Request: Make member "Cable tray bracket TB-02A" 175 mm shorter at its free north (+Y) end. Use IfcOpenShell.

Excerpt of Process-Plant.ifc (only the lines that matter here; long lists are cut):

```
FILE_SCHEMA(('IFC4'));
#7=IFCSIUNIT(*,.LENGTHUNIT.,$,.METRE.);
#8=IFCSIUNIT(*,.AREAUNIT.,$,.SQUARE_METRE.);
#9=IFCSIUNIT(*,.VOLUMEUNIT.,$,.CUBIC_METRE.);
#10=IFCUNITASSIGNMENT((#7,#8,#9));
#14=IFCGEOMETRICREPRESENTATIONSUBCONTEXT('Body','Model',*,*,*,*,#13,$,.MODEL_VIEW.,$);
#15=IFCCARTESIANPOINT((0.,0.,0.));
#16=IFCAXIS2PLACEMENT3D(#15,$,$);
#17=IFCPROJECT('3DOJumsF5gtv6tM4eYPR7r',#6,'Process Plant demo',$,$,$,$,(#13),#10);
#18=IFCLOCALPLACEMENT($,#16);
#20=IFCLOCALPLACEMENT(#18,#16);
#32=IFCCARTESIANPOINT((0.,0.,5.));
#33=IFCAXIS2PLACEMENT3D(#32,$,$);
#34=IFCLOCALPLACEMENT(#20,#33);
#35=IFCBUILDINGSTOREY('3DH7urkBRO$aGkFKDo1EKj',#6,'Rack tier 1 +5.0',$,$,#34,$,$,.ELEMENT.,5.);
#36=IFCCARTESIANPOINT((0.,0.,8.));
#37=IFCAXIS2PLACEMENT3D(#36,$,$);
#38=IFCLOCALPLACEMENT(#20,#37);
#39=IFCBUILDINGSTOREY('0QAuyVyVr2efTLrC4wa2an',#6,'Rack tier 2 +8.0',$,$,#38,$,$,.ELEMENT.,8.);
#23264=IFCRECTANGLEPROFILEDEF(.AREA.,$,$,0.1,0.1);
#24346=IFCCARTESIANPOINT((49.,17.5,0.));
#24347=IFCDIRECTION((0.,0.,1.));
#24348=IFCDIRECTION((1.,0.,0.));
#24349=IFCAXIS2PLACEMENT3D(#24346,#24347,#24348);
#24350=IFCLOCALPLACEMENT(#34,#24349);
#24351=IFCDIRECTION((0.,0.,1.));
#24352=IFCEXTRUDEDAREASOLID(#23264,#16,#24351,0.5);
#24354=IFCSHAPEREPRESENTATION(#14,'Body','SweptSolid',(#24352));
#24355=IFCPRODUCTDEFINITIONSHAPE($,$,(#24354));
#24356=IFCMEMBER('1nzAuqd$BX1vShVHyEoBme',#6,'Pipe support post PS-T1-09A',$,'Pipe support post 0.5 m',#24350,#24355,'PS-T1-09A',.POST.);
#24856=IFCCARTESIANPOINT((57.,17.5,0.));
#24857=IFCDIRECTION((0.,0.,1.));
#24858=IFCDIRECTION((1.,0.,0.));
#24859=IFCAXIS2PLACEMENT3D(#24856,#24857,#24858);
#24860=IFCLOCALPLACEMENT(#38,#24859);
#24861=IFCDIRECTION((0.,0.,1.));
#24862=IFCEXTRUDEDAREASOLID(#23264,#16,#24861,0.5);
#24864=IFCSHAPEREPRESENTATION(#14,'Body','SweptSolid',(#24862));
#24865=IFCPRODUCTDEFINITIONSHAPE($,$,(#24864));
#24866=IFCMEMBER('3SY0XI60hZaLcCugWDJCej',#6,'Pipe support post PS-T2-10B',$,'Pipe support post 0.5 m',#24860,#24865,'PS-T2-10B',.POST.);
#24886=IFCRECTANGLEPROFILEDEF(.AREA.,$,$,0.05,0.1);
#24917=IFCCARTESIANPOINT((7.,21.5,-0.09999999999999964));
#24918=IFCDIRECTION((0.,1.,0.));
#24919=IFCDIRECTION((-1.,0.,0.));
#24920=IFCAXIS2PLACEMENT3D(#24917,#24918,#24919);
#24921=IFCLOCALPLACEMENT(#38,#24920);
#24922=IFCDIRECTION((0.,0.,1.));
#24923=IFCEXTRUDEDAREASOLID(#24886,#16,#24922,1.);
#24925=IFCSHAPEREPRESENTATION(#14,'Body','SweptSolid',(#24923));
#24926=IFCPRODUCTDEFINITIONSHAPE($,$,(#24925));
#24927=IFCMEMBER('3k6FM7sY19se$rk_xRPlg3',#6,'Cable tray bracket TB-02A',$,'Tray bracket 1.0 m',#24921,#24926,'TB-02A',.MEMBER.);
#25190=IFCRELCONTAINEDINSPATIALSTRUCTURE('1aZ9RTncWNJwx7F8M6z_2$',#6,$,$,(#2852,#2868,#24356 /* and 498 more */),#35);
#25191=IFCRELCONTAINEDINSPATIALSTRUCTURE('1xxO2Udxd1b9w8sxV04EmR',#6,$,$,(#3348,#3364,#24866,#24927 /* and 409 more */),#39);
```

```python
import ifcopenshell
import ifcopenshell.util.representation
import ifcopenshell.util.unit

model = ifcopenshell.open("Process-Plant.ifc")
unit_scale = ifcopenshell.util.unit.calculate_unit_scale(model)

member = model.by_guid("3k6FM7sY19se$rk_xRPlg3")
change = -0.175 / unit_scale

# The extrusion runs towards the end named, so only its depth changes.
body = ifcopenshell.util.representation.get_representation(member, "Model", "Body")
solid = body.Items[0]
old_length = solid.Depth
solid.Depth += change

print(f"length {old_length:g} -> {solid.Depth:g}")

model.write("Process-Plant_edited.ifc")
```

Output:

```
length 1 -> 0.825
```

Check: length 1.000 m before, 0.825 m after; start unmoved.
